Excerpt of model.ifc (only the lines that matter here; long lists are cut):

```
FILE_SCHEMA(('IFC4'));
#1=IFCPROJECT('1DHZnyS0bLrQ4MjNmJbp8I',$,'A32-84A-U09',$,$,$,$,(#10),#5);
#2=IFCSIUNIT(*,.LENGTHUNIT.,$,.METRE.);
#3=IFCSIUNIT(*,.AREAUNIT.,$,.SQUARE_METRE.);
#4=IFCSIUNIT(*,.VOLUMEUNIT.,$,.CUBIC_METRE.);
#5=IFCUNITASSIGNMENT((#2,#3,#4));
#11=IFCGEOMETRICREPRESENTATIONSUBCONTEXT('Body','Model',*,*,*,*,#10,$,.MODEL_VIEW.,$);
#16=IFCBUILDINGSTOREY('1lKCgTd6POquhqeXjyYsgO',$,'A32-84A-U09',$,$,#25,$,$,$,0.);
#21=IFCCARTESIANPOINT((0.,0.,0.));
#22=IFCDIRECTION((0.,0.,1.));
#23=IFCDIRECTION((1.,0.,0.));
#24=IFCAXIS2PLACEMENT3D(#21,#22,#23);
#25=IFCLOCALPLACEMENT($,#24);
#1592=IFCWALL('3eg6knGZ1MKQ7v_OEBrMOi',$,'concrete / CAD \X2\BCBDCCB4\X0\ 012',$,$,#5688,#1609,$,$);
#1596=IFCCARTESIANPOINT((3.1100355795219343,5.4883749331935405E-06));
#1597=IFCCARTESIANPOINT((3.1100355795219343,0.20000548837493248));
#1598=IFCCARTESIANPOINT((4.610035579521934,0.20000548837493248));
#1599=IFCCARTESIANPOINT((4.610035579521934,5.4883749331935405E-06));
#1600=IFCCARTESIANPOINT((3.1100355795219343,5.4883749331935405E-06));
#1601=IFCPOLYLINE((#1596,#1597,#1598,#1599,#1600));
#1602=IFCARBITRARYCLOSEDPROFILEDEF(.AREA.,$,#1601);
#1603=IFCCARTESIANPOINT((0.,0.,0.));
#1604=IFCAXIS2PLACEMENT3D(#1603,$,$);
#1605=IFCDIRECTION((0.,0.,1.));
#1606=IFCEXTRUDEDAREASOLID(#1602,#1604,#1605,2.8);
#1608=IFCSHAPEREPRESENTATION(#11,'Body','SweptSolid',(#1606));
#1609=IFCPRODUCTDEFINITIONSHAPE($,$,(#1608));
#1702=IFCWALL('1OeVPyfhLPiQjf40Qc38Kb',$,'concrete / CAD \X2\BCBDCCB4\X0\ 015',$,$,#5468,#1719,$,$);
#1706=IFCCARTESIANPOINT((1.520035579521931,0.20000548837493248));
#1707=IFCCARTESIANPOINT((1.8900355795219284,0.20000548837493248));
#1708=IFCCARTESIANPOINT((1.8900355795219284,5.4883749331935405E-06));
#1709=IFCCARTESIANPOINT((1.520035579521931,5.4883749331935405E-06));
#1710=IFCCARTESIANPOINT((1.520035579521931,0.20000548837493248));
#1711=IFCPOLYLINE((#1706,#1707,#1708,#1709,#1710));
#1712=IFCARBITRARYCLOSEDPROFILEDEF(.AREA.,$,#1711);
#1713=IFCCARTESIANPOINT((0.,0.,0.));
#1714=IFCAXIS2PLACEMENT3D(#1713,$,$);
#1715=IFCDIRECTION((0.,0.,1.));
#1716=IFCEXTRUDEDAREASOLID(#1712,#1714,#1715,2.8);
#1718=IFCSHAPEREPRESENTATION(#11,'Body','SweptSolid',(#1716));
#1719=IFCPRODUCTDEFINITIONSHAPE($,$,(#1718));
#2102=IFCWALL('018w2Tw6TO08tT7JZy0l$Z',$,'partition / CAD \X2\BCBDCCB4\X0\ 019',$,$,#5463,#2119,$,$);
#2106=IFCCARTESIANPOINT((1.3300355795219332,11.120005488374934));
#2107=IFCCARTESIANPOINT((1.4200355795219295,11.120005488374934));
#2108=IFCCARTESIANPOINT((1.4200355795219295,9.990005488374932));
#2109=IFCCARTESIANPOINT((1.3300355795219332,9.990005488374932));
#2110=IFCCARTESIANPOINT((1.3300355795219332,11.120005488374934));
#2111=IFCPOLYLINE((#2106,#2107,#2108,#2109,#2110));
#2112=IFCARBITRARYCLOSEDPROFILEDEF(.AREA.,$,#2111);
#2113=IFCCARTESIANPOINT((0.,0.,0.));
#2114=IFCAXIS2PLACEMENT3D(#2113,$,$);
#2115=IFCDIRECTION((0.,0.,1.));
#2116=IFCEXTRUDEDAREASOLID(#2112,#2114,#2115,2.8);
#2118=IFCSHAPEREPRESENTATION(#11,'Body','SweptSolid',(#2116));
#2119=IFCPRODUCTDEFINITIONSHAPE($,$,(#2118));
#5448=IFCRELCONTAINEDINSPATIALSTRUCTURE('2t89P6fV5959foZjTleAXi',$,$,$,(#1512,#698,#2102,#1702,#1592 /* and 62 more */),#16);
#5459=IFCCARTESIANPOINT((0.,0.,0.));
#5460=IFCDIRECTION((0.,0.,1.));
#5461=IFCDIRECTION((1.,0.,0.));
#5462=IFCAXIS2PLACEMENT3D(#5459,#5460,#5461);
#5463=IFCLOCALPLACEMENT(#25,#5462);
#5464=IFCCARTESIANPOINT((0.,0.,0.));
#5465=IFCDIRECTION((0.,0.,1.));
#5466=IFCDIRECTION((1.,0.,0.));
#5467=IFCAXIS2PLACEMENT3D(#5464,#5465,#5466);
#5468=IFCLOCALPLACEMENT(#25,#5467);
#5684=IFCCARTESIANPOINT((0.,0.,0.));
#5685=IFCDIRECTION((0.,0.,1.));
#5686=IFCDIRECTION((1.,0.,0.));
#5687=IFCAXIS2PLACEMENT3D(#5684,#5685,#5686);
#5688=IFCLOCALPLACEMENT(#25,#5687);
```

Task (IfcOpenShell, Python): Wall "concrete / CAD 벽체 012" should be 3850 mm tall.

```python
import ifcopenshell
import ifcopenshell.geom
import ifcopenshell.util.representation
import ifcopenshell.util.shape
import ifcopenshell.util.unit

model = ifcopenshell.open("model.ifc")
unit_scale = ifcopenshell.util.unit.calculate_unit_scale(model)
settings = ifcopenshell.geom.settings()


def volume(element):
    """Net volume in cubic metres, openings subtracted."""
    shape = ifcopenshell.geom.create_shape(settings, element)
    return ifcopenshell.util.shape.get_volume(shape.geometry)


wall = model.by_id(1592)
before = volume(wall)

body = ifcopenshell.util.representation.get_representation(wall, "Model", "Body")
solid = body.Items[0]
old_height = solid.Depth
solid.Depth = 3.85 / unit_scale
after = volume(wall)

print(f"height {old_height:g} -> {solid.Depth:g}, volume {before:.3f} -> {after:.3f} m3")

model.write("model_v2.ifc")
```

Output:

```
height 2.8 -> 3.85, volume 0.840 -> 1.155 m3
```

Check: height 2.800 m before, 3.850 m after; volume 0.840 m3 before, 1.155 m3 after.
